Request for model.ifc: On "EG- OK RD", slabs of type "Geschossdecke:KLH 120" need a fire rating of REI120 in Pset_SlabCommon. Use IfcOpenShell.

First a look at what the model holds.

```python
import ifcopenshell
import ifcopenshell.util.element

model = ifcopenshell.open("model.ifc")
print(model.schema)
storey = next(s for s in model.by_type("IfcBuildingStorey") if s.Name == "EG- OK RD")
slabs = [e for e in ifcopenshell.util.element.get_decomposition(storey) if e.is_a("IfcSlab")]
seen = {}
for e in slabs:
    element_type = ifcopenshell.util.element.get_type(e)
    key = (element_type.Name if element_type != e and element_type else None, ifcopenshell.util.element.get_pset(e, "Pset_SlabCommon", "FireRating"))
    seen[key] = seen.get(key, 0) + 1
for (name, value), count in sorted(seen.items(), key=str):
    print(count, "x", name, "|", value)
```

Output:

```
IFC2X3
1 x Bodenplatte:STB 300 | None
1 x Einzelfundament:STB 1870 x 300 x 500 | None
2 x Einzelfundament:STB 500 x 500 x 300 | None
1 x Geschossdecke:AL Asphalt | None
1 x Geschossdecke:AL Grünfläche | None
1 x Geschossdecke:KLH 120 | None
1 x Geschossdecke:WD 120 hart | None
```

```python
import ifcopenshell
import ifcopenshell.api.pset
import ifcopenshell.util.element

model = ifcopenshell.open("model.ifc")

storey = next(s for s in model.by_type("IfcBuildingStorey") if s.Name == "EG- OK RD")
slabs = [e for e in ifcopenshell.util.element.get_decomposition(storey) if e.is_a("IfcSlab")]

count = 0
for e in slabs:
    element_type = ifcopenshell.util.element.get_type(e)
    if element_type in (None, e) or element_type.Name != "Geschossdecke:KLH 120":
        continue
    # add_pset returns the element's existing set when there is one.
    pset = ifcopenshell.api.pset.add_pset(model, product=e, name="Pset_SlabCommon")
    ifcopenshell.api.pset.edit_pset(model, pset=pset, properties={"FireRating": "REI120"})
    count += 1

print(count, "slabs updated")

model.write("model_v2.ifc")
```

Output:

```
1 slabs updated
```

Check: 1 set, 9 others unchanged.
